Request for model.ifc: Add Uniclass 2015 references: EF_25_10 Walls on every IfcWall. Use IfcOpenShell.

First a look at what the model holds.

```python
import ifcopenshell

model = ifcopenshell.open("model.ifc")
print(model.schema)
print("classifications:", [c.Name for c in model.by_type("IfcClassification")])
for ifc_class in ("IfcDoor", "IfcRoof", "IfcStair", "IfcWall", "IfcWindow"):
    print(ifc_class, len(model.by_type(ifc_class)))
```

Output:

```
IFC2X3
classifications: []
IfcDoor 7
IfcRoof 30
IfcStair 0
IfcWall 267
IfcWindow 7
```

```python
import ifcopenshell
import ifcopenshell.api.classification

model = ifcopenshell.open("model.ifc")

# IFC2X3 requires Source and Edition and has no link from the project to the system.
system = model.create_entity("IfcClassification", Source="NBS", Edition="2015", Name="Uniclass 2015")

codes = {
    "IfcWall": ("EF_25_10", "Walls"),
}
for ifc_class, (code, name) in codes.items():
    products = model.by_type(ifc_class)
    ifcopenshell.api.classification.add_reference(
        model, products=products, classification=system, identification=code, name=name
    )
    print(code, len(products))

model.write("model-out.ifc")
```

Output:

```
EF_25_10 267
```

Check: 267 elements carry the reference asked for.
